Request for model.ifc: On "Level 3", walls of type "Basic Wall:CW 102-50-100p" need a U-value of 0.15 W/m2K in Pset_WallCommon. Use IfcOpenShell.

First a look at what the model holds.

```python
import ifcopenshell
import ifcopenshell.util.element

model = ifcopenshell.open("model.ifc")
print(model.schema)
storey = next(s for s in model.by_type("IfcBuildingStorey") if s.Name == "Level 3")
walls = [e for e in ifcopenshell.util.element.get_decomposition(storey) if e.is_a("IfcWall")]
seen = {}
for e in walls:
    element_type = ifcopenshell.util.element.get_type(e)
    key = (element_type.Name if element_type != e and element_type else None, ifcopenshell.util.element.get_pset(e, "Pset_WallCommon", "ThermalTransmittance"))
    seen[key] = seen.get(key, 0) + 1
for (name, value), count in sorted(seen.items(), key=str):
    print(count, "x", name, "|", value)
```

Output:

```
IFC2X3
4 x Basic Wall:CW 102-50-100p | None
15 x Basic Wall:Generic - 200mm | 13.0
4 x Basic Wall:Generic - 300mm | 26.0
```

```python
import ifcopenshell
import ifcopenshell.api.pset
import ifcopenshell.util.element

model = ifcopenshell.open("model.ifc")

storey = next(s for s in model.by_type("IfcBuildingStorey") if s.Name == "Level 3")
walls = [e for e in ifcopenshell.util.element.get_decomposition(storey) if e.is_a("IfcWall")]

count = 0
for e in walls:
    element_type = ifcopenshell.util.element.get_type(e)
    if element_type in (None, e) or element_type.Name != "Basic Wall:CW 102-50-100p":
        continue
    # add_pset returns the element's existing set when there is one.
    pset = ifcopenshell.api.pset.add_pset(model, product=e, name="Pset_WallCommon")
    ifcopenshell.api.pset.edit_pset(model, pset=pset, properties={"ThermalTransmittance": 0.15})
    count += 1

print(count, "walls updated")

model.write("model-out.ifc")
```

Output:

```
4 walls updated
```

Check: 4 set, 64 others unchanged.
